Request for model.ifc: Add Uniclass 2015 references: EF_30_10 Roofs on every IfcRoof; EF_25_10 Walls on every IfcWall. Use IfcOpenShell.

First a look at what the model holds.

```python
import ifcopenshell

model = ifcopenshell.open("model.ifc")
print(model.schema)
print("classifications:", [c.Name for c in model.by_type("IfcClassification")])
for ifc_class in ("IfcDoor", "IfcRoof", "IfcStair", "IfcWall", "IfcWindow"):
    print(ifc_class, len(model.by_type(ifc_class)))
```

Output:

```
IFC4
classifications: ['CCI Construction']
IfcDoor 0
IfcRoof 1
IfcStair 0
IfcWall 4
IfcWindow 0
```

```python
import ifcopenshell
import ifcopenshell.api.classification

model = ifcopenshell.open("model.ifc")

system = ifcopenshell.api.classification.add_classification(model, classification="Uniclass 2015")

codes = {
    "IfcRoof": ("EF_30_10", "Roofs"),
    "IfcWall": ("EF_25_10", "Walls"),
}
for ifc_class, (code, name) in codes.items():
    products = model.by_type(ifc_class)
    ifcopenshell.api.classification.add_reference(
        model, products=products, classification=system, identification=code, name=name
    )
    print(code, len(products))

model.write("model_rev.ifc")
```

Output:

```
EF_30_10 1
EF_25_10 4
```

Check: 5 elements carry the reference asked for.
